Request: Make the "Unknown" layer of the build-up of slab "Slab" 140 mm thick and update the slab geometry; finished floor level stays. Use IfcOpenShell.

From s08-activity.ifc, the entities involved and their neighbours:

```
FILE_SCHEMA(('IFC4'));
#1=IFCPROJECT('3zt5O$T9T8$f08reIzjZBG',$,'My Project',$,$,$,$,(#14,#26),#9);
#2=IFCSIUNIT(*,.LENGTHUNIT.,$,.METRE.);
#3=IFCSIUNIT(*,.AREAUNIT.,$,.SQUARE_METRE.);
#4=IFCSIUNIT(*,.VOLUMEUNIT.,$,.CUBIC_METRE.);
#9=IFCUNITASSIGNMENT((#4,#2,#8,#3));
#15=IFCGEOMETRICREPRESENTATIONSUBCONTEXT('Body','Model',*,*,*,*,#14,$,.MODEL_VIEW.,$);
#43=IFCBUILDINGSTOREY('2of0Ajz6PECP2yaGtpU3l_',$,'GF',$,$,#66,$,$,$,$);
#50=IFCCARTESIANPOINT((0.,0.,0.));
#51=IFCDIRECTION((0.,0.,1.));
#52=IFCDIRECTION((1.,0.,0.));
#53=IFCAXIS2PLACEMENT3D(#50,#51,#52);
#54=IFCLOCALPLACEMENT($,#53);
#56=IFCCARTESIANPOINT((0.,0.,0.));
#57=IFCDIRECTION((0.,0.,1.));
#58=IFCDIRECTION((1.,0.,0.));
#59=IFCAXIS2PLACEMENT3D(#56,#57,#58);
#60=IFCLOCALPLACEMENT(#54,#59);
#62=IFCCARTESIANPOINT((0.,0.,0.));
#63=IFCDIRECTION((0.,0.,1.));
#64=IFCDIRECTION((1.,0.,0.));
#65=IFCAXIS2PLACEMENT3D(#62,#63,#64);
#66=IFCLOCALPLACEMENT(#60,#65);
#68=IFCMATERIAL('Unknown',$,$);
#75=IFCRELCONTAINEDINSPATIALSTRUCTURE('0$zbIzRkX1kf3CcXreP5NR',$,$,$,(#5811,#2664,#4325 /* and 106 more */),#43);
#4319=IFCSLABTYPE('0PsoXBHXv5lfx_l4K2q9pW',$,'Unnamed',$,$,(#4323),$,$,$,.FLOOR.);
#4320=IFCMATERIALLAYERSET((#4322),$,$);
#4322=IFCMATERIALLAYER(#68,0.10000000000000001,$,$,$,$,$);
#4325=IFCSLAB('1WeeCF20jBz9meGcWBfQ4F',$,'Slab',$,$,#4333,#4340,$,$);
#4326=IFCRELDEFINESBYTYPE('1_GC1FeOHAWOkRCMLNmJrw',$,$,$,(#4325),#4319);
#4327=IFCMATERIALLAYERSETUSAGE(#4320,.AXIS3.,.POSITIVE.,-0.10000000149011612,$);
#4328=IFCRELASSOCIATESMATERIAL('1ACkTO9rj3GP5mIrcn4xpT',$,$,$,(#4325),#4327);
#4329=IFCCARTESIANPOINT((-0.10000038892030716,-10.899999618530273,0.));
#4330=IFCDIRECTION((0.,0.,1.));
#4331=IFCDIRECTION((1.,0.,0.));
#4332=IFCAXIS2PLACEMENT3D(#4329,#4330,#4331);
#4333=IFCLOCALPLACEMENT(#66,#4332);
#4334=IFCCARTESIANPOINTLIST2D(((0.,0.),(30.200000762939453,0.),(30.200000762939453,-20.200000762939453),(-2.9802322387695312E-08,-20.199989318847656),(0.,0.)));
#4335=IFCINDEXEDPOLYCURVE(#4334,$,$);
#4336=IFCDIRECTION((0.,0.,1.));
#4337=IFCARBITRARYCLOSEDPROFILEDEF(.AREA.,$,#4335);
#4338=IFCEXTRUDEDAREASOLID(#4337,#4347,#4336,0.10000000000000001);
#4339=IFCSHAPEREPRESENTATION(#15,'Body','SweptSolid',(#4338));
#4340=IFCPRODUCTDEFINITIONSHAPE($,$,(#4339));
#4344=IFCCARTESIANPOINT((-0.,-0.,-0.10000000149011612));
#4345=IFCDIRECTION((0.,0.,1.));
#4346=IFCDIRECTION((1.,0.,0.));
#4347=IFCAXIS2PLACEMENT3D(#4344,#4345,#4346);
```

```python
import ifcopenshell
import ifcopenshell.util.element
import ifcopenshell.util.representation
import ifcopenshell.util.unit

model = ifcopenshell.open("s08-activity.ifc")
unit_scale = ifcopenshell.util.unit.calculate_unit_scale(model)

layer_set = model.by_id(4320)
layer = next(l for l in layer_set.MaterialLayers if l.Material and l.Material.Name == "Unknown")
change = 0.14 / unit_scale - layer.LayerThickness
layer.LayerThickness += change

# Geometry does not follow the layer set by itself.
slabs = [e for e in ifcopenshell.util.element.get_elements_by_material(model, layer_set) if e.is_a("IfcSlab")]
for slab in sorted(slabs, key=lambda e: e.id()):
    body = ifcopenshell.util.representation.get_representation(slab, "Model", "Body")
    solid = body.Items[0]
    old_depth = solid.Depth
    solid.Depth += change
    # Extruded upwards: lower the start of the extrusion so the top stays.
    x, y, z = solid.Position.Location.Coordinates
    solid.Position.Location = model.createIfcCartesianPoint((x, y, z - change))
    print(slab.id(), f"{old_depth:g} -> {solid.Depth:g}")

# The layers are counted up from the underside, which has moved.
for usage in {ifcopenshell.util.element.get_material(slab) for slab in slabs}:
    usage.OffsetFromReferenceLine -= change

model.write("s08-activity-out.ifc")
```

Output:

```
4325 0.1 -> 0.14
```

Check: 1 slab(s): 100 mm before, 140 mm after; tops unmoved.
